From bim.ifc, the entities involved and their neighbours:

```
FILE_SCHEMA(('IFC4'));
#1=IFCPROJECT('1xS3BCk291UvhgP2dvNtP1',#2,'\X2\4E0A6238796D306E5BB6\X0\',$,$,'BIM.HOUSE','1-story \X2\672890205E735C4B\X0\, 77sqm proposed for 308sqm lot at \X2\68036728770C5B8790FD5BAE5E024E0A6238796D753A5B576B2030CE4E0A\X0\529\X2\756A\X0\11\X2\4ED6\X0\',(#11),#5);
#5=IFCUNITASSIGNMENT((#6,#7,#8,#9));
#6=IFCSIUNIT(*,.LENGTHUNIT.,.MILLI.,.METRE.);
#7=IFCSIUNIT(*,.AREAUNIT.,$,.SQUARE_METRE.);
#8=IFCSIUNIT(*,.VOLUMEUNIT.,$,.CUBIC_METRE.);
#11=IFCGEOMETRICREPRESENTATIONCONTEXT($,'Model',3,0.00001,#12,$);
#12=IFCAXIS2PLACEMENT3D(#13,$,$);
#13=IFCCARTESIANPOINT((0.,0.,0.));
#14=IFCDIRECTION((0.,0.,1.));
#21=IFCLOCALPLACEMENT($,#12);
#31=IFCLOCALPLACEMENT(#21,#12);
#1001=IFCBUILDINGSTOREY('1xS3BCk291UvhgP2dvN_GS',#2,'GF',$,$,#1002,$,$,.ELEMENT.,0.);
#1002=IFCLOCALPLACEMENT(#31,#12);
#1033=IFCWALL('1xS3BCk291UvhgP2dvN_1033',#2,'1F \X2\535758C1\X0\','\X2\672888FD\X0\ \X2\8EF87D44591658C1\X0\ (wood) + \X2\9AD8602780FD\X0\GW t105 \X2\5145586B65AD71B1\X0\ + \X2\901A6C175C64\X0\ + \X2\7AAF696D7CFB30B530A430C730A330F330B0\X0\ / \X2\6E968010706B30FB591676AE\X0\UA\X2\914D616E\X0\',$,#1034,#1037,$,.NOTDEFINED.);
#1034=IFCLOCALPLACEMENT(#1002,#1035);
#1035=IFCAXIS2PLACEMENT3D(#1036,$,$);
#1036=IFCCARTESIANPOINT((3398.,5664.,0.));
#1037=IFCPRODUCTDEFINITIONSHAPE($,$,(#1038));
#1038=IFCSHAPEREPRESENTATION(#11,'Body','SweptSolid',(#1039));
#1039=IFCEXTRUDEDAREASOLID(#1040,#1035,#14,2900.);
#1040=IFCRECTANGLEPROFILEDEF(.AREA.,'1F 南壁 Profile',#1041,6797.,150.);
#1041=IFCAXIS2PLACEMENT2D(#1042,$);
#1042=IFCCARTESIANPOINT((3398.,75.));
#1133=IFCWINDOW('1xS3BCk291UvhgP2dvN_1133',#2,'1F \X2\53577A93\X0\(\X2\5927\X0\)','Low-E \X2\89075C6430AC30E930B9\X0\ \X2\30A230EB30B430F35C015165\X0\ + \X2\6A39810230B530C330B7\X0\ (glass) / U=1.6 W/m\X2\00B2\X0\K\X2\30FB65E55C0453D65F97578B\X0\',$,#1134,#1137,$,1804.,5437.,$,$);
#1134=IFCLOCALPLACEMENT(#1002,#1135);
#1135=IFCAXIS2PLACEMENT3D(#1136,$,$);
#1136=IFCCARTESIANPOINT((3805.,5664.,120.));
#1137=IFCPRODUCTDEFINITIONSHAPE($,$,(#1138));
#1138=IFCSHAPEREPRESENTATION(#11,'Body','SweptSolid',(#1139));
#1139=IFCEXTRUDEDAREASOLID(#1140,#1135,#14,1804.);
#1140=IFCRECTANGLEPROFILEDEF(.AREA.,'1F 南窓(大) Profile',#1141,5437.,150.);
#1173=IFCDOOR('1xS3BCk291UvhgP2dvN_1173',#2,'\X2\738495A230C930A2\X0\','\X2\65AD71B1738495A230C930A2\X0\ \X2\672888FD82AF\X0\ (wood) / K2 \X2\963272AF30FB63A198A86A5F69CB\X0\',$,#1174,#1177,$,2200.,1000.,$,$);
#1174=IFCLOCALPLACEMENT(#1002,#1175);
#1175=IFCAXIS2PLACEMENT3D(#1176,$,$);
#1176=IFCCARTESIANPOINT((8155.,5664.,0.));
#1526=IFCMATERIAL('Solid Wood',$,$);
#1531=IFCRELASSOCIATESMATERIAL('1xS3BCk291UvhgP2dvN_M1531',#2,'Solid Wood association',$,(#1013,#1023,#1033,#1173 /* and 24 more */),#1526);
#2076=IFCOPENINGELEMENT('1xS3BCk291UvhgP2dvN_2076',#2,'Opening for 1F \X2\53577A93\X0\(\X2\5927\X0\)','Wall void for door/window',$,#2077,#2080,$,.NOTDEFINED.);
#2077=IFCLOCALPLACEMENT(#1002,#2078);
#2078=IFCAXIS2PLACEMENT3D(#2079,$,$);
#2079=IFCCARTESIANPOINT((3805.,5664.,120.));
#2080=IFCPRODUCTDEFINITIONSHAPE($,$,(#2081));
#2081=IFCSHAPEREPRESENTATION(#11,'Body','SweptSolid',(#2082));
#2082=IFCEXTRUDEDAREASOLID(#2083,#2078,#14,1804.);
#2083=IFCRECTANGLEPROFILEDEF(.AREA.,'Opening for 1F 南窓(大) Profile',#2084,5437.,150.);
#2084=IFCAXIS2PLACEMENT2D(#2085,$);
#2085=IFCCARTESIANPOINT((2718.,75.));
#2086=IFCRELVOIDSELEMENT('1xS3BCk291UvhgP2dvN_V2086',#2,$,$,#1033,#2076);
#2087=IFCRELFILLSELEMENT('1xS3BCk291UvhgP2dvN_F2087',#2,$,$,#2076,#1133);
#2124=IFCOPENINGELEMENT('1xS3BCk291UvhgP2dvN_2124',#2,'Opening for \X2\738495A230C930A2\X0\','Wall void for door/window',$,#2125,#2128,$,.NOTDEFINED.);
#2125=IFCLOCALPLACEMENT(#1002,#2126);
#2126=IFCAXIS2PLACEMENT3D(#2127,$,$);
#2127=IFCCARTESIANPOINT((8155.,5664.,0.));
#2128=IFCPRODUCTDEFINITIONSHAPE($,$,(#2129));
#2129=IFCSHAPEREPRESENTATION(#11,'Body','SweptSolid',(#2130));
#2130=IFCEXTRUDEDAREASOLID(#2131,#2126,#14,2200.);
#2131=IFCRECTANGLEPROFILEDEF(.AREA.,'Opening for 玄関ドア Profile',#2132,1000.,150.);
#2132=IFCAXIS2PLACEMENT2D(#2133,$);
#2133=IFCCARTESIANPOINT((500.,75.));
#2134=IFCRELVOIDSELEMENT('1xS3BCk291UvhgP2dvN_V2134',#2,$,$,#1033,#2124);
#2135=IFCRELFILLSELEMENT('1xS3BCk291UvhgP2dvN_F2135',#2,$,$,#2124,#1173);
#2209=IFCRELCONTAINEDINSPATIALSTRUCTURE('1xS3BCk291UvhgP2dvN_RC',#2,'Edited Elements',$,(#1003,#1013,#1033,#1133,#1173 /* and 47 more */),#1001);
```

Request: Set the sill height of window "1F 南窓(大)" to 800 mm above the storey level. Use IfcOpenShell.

```python
import numpy as np
import ifcopenshell
import ifcopenshell.api.geometry
import ifcopenshell.geom
import ifcopenshell.util.element
import ifcopenshell.util.placement
import ifcopenshell.util.shape
import ifcopenshell.util.unit

model = ifcopenshell.open("bim.ifc")
unit_scale = ifcopenshell.util.unit.calculate_unit_scale(model)

window = model.by_guid("1xS3BCk291UvhgP2dvN_1133")
opening = window.FillsVoids[0].RelatingOpeningElement
storey = ifcopenshell.util.element.get_container(window, ifc_class="IfcBuildingStorey")
level = ifcopenshell.util.placement.get_local_placement(storey.ObjectPlacement)[2, 3]

# The opening's origin need not be at the sill, so measure its lowest point.
shape = ifcopenshell.geom.create_shape(ifcopenshell.geom.settings(), opening)
bottom = ifcopenshell.util.shape.get_shape_bottom_elevation(shape, shape.geometry) / unit_scale
dz = level + 0.8 / unit_scale - bottom

shift = np.array([0.0, 0.0, dz])
# The window is not placed relative to its opening, so move both.
for product in (opening, window):
    matrix = ifcopenshell.util.placement.get_local_placement(product.ObjectPlacement)
    matrix[:3, 3] += shift
    ifcopenshell.api.geometry.edit_object_placement(model, product=product, matrix=matrix, is_si=False)

print(f"moved by {dz * unit_scale:+.3f} m")

model.write("bim_v2.ifc")
```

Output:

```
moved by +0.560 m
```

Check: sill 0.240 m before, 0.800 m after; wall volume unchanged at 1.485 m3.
